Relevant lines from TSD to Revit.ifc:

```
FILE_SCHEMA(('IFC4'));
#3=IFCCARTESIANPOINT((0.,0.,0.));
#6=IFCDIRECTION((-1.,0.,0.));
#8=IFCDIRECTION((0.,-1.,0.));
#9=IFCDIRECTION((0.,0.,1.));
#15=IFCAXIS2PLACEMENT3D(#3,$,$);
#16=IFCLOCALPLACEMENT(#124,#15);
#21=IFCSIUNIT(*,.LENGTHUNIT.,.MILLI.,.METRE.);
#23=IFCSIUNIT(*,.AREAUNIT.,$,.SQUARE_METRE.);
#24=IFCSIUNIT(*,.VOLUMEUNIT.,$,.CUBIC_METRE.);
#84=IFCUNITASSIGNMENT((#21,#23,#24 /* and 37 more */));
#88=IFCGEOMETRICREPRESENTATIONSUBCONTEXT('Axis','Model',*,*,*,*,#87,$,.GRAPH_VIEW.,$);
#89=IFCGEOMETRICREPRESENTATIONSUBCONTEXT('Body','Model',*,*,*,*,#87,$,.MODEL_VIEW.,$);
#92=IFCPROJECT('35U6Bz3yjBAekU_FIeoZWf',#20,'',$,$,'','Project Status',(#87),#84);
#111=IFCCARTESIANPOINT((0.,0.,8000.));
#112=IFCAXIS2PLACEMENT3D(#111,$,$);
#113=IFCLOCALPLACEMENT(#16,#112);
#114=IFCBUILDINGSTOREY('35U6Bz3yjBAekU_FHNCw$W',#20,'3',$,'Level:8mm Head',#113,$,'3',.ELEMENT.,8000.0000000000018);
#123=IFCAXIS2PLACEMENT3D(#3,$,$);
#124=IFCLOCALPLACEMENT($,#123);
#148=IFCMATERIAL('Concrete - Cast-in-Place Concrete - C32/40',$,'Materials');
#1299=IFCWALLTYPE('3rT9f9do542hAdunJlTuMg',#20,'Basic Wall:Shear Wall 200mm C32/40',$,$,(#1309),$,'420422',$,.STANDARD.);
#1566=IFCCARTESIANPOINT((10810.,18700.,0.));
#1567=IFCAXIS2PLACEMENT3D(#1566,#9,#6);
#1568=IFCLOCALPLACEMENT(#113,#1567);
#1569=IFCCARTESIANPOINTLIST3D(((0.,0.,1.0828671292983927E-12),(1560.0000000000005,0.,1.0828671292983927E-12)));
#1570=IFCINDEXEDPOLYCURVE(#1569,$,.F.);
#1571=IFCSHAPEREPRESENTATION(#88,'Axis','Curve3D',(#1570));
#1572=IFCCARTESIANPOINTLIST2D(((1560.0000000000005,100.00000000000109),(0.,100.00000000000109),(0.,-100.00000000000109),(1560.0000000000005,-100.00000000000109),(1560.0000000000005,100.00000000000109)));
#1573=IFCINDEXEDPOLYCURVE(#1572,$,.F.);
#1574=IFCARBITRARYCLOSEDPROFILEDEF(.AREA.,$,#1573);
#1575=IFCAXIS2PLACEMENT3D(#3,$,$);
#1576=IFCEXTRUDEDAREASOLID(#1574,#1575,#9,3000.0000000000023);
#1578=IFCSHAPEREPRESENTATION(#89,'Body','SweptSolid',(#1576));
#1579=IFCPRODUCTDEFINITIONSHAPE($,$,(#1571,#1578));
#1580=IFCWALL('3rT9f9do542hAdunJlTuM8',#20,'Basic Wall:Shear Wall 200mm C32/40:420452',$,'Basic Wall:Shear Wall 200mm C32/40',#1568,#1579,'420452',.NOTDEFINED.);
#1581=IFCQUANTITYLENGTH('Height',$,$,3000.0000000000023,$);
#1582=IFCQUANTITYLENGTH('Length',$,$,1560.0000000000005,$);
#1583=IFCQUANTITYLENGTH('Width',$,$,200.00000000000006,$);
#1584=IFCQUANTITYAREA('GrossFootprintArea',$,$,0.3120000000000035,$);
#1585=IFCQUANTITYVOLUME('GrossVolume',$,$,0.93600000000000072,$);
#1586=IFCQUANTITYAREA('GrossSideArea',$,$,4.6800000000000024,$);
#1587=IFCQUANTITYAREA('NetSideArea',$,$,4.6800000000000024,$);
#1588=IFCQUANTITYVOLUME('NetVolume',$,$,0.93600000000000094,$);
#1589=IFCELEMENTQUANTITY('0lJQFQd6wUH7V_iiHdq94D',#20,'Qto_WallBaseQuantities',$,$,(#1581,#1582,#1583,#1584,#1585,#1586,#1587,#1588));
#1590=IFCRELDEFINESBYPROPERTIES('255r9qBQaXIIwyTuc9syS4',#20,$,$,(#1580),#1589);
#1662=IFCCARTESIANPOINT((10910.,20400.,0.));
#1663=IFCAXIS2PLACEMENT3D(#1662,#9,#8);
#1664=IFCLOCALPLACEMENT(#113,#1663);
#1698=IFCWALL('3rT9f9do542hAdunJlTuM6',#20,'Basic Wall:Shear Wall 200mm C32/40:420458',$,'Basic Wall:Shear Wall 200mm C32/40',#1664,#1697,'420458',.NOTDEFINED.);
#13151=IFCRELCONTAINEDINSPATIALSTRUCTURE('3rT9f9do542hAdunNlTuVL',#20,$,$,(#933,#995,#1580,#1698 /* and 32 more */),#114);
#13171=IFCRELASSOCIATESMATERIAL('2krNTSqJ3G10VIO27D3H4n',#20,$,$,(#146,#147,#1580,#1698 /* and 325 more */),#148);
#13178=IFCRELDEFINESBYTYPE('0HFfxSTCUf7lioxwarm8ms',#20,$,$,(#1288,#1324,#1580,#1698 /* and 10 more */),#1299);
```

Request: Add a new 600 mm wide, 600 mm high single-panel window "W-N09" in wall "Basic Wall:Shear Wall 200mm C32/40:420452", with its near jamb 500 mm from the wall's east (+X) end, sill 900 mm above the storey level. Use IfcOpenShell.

```python
import numpy as np
import ifcopenshell
import ifcopenshell.api.feature
import ifcopenshell.api.geometry
import ifcopenshell.api.pset
import ifcopenshell.api.root
import ifcopenshell.api.spatial
import ifcopenshell.geom
import ifcopenshell.util.element
import ifcopenshell.util.placement
import ifcopenshell.util.representation
import ifcopenshell.util.shape
import ifcopenshell.util.unit

model = ifcopenshell.open("TSD to Revit.ifc")
unit_scale = ifcopenshell.util.unit.calculate_unit_scale(model)
area_scale = ifcopenshell.util.unit.calculate_unit_scale(model, "AREAUNIT")
volume_scale = ifcopenshell.util.unit.calculate_unit_scale(model, "VOLUMEUNIT")
settings = ifcopenshell.geom.settings()


def volume(element):
    """Net volume in cubic metres, openings subtracted."""
    shape = ifcopenshell.geom.create_shape(settings, element)
    return ifcopenshell.util.shape.get_volume(shape.geometry)


wall = model.by_guid("3rT9f9do542hAdunJlTuM8")
storey = ifcopenshell.util.element.get_container(wall, ifc_class="IfcBuildingStorey")
context = ifcopenshell.util.representation.get_context(model, "Model", "Body", "MODEL_VIEW")
before = volume(wall)

width, height, from_end, sill = 0.6, 0.6, 0.5, 0.9  # metres

# The wall runs along its own X axis, and the end named is its -X end.
wall_shape = ifcopenshell.geom.create_shape(settings, wall)
x, y, z = ifcopenshell.util.shape.get_vertices(wall_shape.geometry).T
start = x.min() + from_end
face, thickness = float(y.min()), float(y.max() - y.min())
wall_matrix = ifcopenshell.util.placement.get_local_placement(wall.ObjectPlacement)
level = ifcopenshell.util.placement.get_local_placement(storey.ObjectPlacement)[2, 3]


def in_wall(x, y):
    """Placement at x, y metres in the wall's axes, at sill height."""
    matrix = wall_matrix.copy()
    matrix[:, 3] = wall_matrix @ np.array([x / unit_scale, y / unit_scale, 0.0, 1.0])
    matrix[2, 3] = level + sill / unit_scale
    return matrix


# Opening: a box that overshoots both wall faces by 50 mm.
opening = ifcopenshell.api.root.create_entity(model, ifc_class="IfcOpeningElement", predefined_type="OPENING")
box = ifcopenshell.api.geometry.add_wall_representation(
    model, context=context, length=width, height=height, thickness=thickness + 0.1
)
ifcopenshell.api.geometry.assign_representation(model, product=opening, representation=box)
ifcopenshell.api.geometry.edit_object_placement(model, product=opening, matrix=in_wall(start, face - 0.05), is_si=False)
ifcopenshell.api.feature.add_feature(model, feature=opening, element=wall)

window = ifcopenshell.api.root.create_entity(model, ifc_class="IfcWindow", name="W-N09", predefined_type="WINDOW")
window.OverallWidth, window.OverallHeight = width / unit_scale, height / unit_scale
window.PartitioningType = "SINGLE_PANEL"
body = ifcopenshell.api.geometry.add_window_representation(
    model,
    context=context,
    overall_width=window.OverallWidth,
    overall_height=window.OverallHeight,
    partition_type="SINGLE_PANEL",
)
ifcopenshell.api.geometry.assign_representation(model, product=window, representation=body)
ifcopenshell.api.spatial.assign_container(model, products=[window], relating_structure=storey)
ifcopenshell.api.feature.add_filling(model, opening=opening, element=window)

# Centre the window in the wall's thickness.
ifcopenshell.api.geometry.edit_object_placement(model, product=window, matrix=in_wall(start, face), is_si=False)
window_shape = ifcopenshell.geom.create_shape(settings, window)
depth = ifcopenshell.util.shape.get_vertices(window_shape.geometry)[:, 1]
offset = face + thickness / 2 - (depth.min() + depth.max()) / 2
ifcopenshell.api.geometry.edit_object_placement(model, product=window, matrix=in_wall(start, offset), is_si=False)

after = volume(wall)

# Update the wall's stored quantities.
qto = model.by_id(ifcopenshell.util.element.get_pset(wall, "Qto_WallBaseQuantities", should_inherit=False)["id"])
ifcopenshell.api.pset.edit_qto(model, qto=qto, properties={
    "NetSideArea": after / thickness / area_scale,
    "NetVolume": after / volume_scale,
})

print(f"wall volume {before:.3f} -> {after:.3f} m3")

model.write("TSD to Revit_edited.ifc")
```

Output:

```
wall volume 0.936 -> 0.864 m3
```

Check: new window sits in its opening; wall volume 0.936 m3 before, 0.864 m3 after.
